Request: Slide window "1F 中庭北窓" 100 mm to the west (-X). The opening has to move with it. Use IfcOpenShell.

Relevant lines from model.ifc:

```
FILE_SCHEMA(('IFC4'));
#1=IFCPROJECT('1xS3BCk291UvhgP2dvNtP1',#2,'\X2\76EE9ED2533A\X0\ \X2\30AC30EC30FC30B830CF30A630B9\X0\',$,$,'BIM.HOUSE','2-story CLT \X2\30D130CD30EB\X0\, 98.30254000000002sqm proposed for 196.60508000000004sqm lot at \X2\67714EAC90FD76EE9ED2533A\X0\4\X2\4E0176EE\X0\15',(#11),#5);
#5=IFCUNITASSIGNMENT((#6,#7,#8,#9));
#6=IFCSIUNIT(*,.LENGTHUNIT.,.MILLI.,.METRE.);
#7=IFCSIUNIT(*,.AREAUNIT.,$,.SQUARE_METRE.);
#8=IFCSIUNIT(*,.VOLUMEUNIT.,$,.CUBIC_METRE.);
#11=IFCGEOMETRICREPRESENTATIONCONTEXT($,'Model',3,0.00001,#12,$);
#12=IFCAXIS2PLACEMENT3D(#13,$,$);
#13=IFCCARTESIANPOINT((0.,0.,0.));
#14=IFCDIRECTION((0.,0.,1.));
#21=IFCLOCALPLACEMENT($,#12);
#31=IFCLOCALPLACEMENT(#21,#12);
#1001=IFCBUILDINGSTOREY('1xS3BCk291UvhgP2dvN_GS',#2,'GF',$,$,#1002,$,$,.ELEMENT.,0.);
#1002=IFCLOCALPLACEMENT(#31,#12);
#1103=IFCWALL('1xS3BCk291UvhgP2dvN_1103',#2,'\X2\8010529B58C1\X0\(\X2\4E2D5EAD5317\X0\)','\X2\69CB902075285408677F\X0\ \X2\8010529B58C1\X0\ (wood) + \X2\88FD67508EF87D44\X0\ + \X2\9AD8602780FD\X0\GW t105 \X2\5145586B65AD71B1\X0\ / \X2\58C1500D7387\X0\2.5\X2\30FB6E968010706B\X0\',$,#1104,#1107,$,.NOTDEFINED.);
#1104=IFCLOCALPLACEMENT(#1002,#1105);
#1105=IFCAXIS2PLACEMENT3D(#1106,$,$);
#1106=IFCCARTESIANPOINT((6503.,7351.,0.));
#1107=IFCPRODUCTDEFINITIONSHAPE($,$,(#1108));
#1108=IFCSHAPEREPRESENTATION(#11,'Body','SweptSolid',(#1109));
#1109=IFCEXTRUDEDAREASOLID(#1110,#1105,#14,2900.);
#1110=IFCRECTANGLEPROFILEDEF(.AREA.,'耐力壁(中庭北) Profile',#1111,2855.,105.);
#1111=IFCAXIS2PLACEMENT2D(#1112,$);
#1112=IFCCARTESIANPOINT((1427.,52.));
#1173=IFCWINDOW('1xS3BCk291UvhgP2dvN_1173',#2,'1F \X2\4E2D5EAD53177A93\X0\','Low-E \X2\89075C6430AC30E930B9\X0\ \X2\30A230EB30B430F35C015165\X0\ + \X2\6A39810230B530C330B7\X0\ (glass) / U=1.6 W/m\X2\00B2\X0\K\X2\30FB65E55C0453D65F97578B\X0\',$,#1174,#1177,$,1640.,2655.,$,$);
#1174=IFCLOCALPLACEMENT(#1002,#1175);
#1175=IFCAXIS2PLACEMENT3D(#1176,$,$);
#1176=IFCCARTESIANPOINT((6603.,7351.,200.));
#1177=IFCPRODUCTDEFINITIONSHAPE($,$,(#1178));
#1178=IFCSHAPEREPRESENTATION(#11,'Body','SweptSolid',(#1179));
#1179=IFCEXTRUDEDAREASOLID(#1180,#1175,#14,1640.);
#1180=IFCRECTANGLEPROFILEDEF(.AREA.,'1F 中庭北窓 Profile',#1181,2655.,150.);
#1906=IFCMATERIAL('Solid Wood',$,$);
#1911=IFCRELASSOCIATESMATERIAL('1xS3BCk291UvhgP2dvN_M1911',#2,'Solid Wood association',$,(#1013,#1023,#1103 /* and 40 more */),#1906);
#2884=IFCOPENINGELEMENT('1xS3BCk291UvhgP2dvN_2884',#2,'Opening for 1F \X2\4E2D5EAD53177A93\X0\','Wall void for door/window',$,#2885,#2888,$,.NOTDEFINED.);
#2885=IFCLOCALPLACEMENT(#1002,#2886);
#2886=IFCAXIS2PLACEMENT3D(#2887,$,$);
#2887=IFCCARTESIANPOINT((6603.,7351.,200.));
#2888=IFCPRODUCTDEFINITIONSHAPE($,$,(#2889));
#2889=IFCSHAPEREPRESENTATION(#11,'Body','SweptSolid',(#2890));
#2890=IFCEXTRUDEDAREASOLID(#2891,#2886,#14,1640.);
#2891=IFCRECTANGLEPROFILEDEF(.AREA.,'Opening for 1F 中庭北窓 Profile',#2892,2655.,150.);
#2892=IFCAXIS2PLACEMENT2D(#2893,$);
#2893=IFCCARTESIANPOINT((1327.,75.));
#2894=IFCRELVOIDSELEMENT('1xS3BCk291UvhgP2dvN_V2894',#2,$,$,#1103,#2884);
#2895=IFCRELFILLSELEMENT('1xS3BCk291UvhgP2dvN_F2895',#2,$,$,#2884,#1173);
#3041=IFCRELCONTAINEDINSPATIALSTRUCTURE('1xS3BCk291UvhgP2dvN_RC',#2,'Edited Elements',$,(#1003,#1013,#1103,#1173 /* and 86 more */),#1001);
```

```python
import ifcopenshell
import ifcopenshell.api.geometry
import ifcopenshell.util.placement
import ifcopenshell.util.unit

model = ifcopenshell.open("model.ifc")
unit_scale = ifcopenshell.util.unit.calculate_unit_scale(model)

window = model.by_guid("1xS3BCk291UvhgP2dvN_1173")
opening = window.FillsVoids[0].RelatingOpeningElement
wall = opening.VoidsElements[0].RelatingBuildingElement

wall_matrix = ifcopenshell.util.placement.get_local_placement(wall.ObjectPlacement)
shift = wall_matrix[:3, 0] * -0.1 / unit_scale
before = ifcopenshell.util.placement.get_local_placement(window.ObjectPlacement)[:3, 3].copy()

# The window is not placed relative to its opening, so move both.
for product in (opening, window):
    matrix = ifcopenshell.util.placement.get_local_placement(product.ObjectPlacement)
    matrix[:3, 3] += shift
    ifcopenshell.api.geometry.edit_object_placement(model, product=product, matrix=matrix, is_si=False)

after = ifcopenshell.util.placement.get_local_placement(window.ObjectPlacement)[:3, 3]
print("window moved by", (after - before).round(3) + 0.0)

model.write("model_edited.ifc")
```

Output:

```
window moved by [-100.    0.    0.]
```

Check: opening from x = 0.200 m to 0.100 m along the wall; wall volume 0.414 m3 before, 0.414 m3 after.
